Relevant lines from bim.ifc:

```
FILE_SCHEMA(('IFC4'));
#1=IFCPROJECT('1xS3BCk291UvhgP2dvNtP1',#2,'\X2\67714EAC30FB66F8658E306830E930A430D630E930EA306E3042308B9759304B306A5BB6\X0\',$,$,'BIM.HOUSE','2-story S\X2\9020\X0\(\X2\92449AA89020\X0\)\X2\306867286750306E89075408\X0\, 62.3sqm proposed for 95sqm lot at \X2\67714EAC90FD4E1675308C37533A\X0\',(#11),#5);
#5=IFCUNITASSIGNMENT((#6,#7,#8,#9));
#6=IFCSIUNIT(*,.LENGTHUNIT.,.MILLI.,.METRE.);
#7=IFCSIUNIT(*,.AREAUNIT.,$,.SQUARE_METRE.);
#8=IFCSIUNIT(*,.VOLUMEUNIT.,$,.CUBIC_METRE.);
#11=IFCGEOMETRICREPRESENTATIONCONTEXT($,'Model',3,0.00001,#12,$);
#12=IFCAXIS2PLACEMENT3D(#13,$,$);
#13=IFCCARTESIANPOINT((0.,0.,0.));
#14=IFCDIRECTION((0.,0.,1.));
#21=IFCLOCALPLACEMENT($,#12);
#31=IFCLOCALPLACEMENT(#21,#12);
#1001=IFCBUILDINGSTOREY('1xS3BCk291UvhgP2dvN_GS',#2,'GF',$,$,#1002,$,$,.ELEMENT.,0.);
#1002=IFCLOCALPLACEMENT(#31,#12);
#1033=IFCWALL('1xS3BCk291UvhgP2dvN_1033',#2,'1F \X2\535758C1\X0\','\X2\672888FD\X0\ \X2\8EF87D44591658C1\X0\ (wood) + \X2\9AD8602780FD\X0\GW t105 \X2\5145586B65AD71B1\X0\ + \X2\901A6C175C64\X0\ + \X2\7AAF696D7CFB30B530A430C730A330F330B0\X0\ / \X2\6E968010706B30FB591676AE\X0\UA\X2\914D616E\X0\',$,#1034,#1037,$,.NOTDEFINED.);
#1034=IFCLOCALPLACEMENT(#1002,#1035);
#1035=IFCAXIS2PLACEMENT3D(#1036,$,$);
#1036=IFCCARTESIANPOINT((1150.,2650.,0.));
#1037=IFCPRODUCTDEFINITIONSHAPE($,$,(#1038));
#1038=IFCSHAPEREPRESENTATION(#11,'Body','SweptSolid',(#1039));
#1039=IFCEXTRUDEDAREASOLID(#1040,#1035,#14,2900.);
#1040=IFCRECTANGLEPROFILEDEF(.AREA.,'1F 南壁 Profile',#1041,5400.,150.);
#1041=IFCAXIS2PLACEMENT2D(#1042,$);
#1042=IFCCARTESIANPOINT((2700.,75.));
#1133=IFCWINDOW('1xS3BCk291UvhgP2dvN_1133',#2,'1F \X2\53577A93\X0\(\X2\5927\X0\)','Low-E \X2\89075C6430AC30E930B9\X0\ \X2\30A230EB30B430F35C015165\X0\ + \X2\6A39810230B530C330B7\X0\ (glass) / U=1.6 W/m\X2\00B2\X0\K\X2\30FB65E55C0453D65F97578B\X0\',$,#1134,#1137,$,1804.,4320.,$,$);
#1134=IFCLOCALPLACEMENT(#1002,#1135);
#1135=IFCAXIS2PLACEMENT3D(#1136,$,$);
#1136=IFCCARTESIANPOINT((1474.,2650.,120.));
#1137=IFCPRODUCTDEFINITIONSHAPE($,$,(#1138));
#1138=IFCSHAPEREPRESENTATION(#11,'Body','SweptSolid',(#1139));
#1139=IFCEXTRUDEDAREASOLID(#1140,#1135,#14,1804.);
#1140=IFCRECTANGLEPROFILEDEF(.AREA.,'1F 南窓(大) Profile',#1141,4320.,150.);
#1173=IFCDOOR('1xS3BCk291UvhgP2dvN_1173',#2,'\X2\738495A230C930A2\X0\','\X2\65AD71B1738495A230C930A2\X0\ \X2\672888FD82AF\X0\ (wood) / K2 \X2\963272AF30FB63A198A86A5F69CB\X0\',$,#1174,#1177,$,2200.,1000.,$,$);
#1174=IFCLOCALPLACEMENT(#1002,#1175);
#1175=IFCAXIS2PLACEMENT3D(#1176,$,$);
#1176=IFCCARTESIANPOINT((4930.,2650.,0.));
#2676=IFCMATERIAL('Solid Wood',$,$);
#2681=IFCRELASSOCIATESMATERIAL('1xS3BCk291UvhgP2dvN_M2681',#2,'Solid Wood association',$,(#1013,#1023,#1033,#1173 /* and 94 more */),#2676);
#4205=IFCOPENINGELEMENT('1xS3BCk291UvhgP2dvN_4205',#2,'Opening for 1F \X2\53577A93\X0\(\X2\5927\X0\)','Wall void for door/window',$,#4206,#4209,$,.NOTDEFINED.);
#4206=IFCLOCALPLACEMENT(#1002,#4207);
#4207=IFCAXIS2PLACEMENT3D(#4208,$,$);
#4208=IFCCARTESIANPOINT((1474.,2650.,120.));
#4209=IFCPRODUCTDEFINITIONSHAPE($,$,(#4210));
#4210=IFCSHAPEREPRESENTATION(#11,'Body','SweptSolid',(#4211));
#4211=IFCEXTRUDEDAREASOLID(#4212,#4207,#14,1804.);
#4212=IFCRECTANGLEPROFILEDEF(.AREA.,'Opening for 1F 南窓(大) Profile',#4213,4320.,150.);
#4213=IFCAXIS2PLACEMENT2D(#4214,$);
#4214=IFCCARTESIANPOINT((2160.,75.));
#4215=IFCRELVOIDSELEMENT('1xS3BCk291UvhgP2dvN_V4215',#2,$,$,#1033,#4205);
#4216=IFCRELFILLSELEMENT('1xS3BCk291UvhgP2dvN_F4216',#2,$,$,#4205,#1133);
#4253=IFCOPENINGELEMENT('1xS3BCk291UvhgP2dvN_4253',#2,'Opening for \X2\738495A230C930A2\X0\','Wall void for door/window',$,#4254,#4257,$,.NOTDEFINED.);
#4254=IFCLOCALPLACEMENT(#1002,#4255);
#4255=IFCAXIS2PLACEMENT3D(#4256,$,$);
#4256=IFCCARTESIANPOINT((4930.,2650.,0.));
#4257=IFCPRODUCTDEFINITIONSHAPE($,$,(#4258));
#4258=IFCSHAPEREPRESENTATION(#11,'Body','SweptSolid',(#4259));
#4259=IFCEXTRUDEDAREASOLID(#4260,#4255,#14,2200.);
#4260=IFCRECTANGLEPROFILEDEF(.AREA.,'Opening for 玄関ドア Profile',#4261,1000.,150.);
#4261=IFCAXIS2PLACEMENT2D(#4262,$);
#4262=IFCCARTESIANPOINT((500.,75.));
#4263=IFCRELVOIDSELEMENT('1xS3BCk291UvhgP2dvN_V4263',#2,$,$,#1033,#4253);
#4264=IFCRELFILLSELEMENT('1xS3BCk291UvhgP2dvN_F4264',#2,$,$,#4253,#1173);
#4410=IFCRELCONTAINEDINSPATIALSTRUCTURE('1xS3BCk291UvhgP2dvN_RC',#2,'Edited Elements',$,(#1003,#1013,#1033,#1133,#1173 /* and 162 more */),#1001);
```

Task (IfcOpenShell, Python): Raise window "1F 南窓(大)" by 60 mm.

```python
import numpy as np
import ifcopenshell
import ifcopenshell.api.geometry
import ifcopenshell.util.placement
import ifcopenshell.util.unit

model = ifcopenshell.open("bim.ifc")
unit_scale = ifcopenshell.util.unit.calculate_unit_scale(model)

window = model.by_guid("1xS3BCk291UvhgP2dvN_1133")
opening = window.FillsVoids[0].RelatingOpeningElement
dz = 0.06 / unit_scale

shift = np.array([0.0, 0.0, dz])
# The window is not placed relative to its opening, so move both.
for product in (opening, window):
    matrix = ifcopenshell.util.placement.get_local_placement(product.ObjectPlacement)
    matrix[:3, 3] += shift
    ifcopenshell.api.geometry.edit_object_placement(model, product=product, matrix=matrix, is_si=False)

print(f"moved by {dz * unit_scale:+.3f} m")

model.write("bim-out.ifc")
```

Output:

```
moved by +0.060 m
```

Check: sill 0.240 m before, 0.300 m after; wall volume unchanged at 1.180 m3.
